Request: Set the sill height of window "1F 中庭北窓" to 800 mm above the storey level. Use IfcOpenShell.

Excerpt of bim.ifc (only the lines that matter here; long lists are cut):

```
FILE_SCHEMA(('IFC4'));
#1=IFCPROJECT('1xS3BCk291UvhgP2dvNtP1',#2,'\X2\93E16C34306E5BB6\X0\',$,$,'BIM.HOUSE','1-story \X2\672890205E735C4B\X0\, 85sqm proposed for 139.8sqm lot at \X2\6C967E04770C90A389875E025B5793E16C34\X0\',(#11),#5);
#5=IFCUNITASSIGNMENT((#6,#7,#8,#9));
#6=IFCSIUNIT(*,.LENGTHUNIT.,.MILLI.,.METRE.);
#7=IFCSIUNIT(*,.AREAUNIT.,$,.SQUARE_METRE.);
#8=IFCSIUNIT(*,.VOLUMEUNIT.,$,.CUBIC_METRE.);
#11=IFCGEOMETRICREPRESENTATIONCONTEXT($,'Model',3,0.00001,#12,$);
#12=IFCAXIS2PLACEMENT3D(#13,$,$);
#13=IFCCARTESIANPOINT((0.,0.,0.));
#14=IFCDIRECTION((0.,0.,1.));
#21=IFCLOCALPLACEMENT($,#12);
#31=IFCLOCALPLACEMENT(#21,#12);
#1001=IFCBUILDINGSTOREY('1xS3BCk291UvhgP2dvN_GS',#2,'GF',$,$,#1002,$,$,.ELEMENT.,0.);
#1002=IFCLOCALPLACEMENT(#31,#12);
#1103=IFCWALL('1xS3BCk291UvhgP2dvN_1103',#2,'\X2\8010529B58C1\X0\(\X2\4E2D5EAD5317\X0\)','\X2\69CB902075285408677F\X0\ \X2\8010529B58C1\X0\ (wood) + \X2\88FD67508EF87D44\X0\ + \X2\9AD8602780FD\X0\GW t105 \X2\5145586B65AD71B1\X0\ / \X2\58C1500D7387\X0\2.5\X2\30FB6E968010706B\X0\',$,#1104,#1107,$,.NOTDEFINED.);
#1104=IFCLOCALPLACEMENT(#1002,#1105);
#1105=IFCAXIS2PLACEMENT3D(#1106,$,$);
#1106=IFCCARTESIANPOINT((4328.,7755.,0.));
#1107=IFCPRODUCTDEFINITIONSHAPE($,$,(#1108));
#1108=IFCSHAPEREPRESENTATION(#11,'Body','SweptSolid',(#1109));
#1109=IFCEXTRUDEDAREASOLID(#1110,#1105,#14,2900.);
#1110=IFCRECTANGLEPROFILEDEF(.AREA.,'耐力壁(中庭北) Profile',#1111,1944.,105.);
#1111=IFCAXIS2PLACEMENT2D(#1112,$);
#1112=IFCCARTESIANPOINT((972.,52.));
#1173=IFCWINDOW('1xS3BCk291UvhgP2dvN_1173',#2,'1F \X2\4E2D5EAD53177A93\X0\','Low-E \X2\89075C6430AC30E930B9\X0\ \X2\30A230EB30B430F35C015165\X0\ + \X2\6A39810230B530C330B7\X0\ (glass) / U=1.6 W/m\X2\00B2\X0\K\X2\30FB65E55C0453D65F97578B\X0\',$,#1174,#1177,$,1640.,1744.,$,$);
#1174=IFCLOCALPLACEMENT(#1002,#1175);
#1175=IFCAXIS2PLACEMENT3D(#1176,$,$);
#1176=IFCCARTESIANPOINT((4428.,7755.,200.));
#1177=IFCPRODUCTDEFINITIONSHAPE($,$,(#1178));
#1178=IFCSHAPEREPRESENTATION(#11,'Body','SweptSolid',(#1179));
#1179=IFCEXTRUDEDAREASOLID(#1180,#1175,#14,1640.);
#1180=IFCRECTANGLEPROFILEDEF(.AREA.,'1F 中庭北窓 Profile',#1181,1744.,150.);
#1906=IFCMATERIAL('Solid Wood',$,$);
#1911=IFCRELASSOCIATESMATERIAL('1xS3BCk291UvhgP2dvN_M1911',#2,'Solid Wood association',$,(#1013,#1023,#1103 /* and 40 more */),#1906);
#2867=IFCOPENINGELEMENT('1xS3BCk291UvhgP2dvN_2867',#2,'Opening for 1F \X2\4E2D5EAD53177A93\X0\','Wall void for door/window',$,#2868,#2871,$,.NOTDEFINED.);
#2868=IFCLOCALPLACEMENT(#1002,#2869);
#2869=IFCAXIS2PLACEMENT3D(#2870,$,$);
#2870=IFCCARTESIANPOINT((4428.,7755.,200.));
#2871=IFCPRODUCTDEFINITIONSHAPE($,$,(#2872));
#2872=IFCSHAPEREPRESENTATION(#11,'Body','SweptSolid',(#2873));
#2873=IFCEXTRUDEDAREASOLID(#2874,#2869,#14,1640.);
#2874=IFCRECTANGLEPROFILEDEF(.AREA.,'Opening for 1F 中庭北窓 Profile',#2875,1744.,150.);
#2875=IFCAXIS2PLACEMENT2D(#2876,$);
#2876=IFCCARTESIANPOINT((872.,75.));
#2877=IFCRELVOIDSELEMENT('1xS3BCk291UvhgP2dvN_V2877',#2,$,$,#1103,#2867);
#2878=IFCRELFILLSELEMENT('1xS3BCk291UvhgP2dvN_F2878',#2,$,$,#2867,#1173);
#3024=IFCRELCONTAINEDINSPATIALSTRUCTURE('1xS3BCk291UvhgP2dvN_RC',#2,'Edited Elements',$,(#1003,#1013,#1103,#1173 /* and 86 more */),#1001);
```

```python
import numpy as np
import ifcopenshell
import ifcopenshell.api.geometry
import ifcopenshell.geom
import ifcopenshell.util.element
import ifcopenshell.util.placement
import ifcopenshell.util.shape
import ifcopenshell.util.unit

model = ifcopenshell.open("bim.ifc")
unit_scale = ifcopenshell.util.unit.calculate_unit_scale(model)

window = model.by_guid("1xS3BCk291UvhgP2dvN_1173")
opening = window.FillsVoids[0].RelatingOpeningElement
storey = ifcopenshell.util.element.get_container(window, ifc_class="IfcBuildingStorey")
level = ifcopenshell.util.placement.get_local_placement(storey.ObjectPlacement)[2, 3]

# The opening's origin need not be at the sill, so measure its lowest point.
shape = ifcopenshell.geom.create_shape(ifcopenshell.geom.settings(), opening)
bottom = ifcopenshell.util.shape.get_shape_bottom_elevation(shape, shape.geometry) / unit_scale
dz = level + 0.8 / unit_scale - bottom

shift = np.array([0.0, 0.0, dz])
# The window is not placed relative to its opening, so move both.
for product in (opening, window):
    matrix = ifcopenshell.util.placement.get_local_placement(product.ObjectPlacement)
    matrix[:3, 3] += shift
    ifcopenshell.api.geometry.edit_object_placement(model, product=product, matrix=matrix, is_si=False)

print(f"moved by {dz * unit_scale:+.3f} m")

model.write("bim-out.ifc")
```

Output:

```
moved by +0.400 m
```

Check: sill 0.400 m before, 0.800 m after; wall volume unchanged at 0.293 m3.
